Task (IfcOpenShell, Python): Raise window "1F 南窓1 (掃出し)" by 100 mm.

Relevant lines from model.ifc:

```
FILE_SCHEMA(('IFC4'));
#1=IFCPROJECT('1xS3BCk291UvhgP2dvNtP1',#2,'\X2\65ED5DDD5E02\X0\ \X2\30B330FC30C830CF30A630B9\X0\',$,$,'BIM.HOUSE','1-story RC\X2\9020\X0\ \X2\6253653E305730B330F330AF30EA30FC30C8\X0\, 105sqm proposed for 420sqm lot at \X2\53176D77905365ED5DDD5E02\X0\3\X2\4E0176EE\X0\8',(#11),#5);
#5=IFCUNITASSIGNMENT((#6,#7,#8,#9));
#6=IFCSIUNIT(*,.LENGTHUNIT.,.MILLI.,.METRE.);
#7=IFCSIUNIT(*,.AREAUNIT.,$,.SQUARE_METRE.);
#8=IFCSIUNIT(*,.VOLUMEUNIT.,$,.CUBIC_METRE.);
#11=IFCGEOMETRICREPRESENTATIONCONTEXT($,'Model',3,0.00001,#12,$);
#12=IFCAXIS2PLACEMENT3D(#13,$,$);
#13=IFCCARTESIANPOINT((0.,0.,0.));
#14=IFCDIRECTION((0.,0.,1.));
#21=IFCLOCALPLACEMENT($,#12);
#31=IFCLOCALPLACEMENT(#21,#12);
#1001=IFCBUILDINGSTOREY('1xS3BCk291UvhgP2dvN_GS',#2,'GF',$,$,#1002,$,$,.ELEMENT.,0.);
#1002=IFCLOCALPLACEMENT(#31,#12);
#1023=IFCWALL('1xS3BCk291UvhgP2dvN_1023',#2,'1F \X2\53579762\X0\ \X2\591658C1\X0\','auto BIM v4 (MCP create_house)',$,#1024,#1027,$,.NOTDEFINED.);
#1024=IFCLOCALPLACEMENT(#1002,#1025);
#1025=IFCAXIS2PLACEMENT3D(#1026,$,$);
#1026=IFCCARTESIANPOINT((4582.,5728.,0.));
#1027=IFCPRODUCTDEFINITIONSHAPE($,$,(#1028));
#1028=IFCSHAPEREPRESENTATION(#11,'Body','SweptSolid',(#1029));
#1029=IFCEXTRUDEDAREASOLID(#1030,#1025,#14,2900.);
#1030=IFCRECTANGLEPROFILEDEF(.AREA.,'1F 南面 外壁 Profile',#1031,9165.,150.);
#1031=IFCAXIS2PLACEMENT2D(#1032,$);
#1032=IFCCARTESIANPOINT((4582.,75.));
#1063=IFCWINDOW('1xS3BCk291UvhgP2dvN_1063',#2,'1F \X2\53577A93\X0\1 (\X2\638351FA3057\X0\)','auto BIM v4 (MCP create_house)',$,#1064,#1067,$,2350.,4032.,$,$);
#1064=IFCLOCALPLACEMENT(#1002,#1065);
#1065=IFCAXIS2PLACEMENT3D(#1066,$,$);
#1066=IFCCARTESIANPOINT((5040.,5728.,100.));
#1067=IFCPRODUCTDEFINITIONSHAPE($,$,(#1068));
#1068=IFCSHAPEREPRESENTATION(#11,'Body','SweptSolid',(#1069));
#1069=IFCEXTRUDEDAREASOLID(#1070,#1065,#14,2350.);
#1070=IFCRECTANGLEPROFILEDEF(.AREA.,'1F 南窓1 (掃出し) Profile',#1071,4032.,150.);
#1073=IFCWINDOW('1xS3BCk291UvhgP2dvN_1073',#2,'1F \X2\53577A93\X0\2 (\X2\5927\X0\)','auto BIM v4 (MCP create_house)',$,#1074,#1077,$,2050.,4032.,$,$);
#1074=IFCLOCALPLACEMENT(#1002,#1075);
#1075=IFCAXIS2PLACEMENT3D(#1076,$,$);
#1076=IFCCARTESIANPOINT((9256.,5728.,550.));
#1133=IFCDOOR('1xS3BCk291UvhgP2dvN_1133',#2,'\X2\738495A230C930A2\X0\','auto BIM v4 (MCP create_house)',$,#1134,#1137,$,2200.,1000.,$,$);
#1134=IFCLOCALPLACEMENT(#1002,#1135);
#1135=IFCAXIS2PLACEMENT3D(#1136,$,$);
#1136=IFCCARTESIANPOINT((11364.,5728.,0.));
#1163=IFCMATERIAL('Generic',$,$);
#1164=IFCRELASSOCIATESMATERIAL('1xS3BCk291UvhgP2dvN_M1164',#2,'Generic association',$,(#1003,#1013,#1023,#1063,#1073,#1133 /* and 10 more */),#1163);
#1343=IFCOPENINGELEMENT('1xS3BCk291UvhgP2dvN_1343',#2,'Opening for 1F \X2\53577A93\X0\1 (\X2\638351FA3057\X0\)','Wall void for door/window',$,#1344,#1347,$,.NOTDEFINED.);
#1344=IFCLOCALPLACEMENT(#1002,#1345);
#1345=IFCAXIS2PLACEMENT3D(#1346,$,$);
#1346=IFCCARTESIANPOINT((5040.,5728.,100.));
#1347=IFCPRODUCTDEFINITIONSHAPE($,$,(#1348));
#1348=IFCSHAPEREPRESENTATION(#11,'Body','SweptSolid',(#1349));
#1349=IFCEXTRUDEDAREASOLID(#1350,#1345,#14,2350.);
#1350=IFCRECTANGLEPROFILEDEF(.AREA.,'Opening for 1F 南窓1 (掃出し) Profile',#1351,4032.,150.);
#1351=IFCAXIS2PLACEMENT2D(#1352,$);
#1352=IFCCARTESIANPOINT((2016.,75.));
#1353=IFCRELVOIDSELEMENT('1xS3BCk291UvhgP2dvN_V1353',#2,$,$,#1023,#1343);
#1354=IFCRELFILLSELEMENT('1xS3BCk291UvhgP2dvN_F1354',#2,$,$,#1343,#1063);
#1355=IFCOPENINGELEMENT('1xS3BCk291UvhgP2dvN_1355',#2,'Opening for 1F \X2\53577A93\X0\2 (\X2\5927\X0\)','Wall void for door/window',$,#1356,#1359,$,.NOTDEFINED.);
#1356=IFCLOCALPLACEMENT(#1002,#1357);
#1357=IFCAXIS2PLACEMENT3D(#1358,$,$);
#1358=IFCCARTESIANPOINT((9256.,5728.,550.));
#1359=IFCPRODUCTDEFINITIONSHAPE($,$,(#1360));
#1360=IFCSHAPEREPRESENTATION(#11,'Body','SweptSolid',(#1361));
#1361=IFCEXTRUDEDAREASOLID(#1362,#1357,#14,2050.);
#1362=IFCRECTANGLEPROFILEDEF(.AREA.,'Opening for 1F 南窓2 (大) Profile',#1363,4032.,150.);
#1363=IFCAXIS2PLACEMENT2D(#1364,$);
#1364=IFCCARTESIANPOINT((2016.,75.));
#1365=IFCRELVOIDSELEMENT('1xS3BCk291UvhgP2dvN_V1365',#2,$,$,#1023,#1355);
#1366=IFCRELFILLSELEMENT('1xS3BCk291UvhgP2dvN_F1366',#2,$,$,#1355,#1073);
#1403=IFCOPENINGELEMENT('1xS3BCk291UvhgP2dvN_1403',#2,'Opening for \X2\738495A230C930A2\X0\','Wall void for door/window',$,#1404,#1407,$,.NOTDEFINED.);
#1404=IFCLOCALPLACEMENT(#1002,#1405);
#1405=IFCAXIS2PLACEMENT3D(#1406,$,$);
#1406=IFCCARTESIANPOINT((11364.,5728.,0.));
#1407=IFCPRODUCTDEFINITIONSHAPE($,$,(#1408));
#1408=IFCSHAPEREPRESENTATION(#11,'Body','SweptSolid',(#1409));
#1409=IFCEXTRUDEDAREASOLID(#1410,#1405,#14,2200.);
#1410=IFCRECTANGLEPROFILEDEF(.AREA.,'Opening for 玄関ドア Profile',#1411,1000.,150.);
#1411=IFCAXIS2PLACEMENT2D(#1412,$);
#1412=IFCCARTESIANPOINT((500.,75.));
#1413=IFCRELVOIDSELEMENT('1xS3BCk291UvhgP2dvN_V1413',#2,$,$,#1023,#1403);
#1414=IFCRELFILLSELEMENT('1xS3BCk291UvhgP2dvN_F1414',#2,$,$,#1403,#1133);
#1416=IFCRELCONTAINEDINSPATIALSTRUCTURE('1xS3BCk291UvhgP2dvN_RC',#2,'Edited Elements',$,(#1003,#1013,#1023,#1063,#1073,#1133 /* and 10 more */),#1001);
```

```python
import numpy as np
import ifcopenshell
import ifcopenshell.api.geometry
import ifcopenshell.util.placement
import ifcopenshell.util.unit

model = ifcopenshell.open("model.ifc")
unit_scale = ifcopenshell.util.unit.calculate_unit_scale(model)

window = model.by_id(1063)
opening = window.FillsVoids[0].RelatingOpeningElement
dz = 0.1 / unit_scale

shift = np.array([0.0, 0.0, dz])
# The window is not placed relative to its opening, so move both.
for product in (opening, window):
    matrix = ifcopenshell.util.placement.get_local_placement(product.ObjectPlacement)
    matrix[:3, 3] += shift
    ifcopenshell.api.geometry.edit_object_placement(model, product=product, matrix=matrix, is_si=False)

print(f"moved by {dz * unit_scale:+.3f} m")

model.write("model-out.ifc")
```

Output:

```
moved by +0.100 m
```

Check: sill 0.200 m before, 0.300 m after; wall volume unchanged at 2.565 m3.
